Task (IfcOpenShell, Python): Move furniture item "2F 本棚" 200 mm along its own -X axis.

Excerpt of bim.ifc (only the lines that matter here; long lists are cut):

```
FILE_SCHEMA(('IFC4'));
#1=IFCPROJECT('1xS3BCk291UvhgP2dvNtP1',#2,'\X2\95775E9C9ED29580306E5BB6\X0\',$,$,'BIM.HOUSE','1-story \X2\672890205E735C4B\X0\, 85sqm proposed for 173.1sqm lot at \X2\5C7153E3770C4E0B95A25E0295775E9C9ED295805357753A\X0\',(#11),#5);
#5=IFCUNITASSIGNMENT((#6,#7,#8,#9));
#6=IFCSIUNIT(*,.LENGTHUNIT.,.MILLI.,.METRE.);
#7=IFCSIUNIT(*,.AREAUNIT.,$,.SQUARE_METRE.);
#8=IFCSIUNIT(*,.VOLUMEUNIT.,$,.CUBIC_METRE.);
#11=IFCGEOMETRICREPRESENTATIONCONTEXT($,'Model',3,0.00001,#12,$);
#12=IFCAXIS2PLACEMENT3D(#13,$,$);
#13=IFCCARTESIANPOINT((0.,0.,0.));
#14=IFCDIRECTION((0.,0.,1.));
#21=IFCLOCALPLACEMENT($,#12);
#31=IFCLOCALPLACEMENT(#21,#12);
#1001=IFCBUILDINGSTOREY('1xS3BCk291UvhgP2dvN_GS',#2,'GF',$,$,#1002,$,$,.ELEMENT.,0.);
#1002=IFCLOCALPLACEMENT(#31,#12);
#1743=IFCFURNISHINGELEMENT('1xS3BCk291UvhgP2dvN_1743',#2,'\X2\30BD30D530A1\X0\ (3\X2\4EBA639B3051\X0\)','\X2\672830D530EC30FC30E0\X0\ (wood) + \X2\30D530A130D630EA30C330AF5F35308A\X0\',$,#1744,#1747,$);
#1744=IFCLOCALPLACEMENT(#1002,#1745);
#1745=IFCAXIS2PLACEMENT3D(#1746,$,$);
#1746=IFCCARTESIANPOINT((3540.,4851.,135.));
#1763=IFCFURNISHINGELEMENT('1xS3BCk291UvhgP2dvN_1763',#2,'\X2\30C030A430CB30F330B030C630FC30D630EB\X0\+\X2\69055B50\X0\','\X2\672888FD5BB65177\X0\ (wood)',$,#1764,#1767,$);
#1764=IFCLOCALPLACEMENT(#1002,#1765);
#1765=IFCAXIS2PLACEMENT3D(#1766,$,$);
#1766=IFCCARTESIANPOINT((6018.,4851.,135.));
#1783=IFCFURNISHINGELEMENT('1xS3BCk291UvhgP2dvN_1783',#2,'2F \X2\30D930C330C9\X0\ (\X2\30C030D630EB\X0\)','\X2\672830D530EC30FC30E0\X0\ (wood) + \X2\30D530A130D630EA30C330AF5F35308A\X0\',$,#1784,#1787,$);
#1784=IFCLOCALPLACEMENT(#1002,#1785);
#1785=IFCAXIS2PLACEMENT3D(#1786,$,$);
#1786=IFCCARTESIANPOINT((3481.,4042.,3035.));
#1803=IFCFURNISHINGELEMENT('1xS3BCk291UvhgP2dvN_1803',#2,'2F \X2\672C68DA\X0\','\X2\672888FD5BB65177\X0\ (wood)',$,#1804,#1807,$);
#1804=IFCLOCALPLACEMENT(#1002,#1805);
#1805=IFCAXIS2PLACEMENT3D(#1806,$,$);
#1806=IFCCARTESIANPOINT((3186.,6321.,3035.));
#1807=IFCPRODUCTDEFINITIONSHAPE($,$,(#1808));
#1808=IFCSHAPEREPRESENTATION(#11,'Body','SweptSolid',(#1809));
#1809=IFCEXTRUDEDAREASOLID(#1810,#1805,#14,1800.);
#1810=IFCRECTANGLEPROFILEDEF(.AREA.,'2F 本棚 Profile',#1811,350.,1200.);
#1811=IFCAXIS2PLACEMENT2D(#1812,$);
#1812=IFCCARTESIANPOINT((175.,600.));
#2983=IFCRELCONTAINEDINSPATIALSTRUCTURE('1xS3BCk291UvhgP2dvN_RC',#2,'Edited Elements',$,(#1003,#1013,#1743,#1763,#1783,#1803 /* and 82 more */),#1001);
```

```python
import ifcopenshell
import ifcopenshell.api.geometry
import ifcopenshell.util.placement

model = ifcopenshell.open("bim.ifc")

item = model.by_id(1803)
matrix = ifcopenshell.util.placement.get_local_placement(item.ObjectPlacement)
matrix[:3, 3] -= matrix[:3, 0] * 200.0
ifcopenshell.api.geometry.edit_object_placement(model, product=item, matrix=matrix, is_si=False)

print(ifcopenshell.util.placement.get_local_placement(item.ObjectPlacement).round(3) + 0.0)

model.write("bim_rev.ifc")
```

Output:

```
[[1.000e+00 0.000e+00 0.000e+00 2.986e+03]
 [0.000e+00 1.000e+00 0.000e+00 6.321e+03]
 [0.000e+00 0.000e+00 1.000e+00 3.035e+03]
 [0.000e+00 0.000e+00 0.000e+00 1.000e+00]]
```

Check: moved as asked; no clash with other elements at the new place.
